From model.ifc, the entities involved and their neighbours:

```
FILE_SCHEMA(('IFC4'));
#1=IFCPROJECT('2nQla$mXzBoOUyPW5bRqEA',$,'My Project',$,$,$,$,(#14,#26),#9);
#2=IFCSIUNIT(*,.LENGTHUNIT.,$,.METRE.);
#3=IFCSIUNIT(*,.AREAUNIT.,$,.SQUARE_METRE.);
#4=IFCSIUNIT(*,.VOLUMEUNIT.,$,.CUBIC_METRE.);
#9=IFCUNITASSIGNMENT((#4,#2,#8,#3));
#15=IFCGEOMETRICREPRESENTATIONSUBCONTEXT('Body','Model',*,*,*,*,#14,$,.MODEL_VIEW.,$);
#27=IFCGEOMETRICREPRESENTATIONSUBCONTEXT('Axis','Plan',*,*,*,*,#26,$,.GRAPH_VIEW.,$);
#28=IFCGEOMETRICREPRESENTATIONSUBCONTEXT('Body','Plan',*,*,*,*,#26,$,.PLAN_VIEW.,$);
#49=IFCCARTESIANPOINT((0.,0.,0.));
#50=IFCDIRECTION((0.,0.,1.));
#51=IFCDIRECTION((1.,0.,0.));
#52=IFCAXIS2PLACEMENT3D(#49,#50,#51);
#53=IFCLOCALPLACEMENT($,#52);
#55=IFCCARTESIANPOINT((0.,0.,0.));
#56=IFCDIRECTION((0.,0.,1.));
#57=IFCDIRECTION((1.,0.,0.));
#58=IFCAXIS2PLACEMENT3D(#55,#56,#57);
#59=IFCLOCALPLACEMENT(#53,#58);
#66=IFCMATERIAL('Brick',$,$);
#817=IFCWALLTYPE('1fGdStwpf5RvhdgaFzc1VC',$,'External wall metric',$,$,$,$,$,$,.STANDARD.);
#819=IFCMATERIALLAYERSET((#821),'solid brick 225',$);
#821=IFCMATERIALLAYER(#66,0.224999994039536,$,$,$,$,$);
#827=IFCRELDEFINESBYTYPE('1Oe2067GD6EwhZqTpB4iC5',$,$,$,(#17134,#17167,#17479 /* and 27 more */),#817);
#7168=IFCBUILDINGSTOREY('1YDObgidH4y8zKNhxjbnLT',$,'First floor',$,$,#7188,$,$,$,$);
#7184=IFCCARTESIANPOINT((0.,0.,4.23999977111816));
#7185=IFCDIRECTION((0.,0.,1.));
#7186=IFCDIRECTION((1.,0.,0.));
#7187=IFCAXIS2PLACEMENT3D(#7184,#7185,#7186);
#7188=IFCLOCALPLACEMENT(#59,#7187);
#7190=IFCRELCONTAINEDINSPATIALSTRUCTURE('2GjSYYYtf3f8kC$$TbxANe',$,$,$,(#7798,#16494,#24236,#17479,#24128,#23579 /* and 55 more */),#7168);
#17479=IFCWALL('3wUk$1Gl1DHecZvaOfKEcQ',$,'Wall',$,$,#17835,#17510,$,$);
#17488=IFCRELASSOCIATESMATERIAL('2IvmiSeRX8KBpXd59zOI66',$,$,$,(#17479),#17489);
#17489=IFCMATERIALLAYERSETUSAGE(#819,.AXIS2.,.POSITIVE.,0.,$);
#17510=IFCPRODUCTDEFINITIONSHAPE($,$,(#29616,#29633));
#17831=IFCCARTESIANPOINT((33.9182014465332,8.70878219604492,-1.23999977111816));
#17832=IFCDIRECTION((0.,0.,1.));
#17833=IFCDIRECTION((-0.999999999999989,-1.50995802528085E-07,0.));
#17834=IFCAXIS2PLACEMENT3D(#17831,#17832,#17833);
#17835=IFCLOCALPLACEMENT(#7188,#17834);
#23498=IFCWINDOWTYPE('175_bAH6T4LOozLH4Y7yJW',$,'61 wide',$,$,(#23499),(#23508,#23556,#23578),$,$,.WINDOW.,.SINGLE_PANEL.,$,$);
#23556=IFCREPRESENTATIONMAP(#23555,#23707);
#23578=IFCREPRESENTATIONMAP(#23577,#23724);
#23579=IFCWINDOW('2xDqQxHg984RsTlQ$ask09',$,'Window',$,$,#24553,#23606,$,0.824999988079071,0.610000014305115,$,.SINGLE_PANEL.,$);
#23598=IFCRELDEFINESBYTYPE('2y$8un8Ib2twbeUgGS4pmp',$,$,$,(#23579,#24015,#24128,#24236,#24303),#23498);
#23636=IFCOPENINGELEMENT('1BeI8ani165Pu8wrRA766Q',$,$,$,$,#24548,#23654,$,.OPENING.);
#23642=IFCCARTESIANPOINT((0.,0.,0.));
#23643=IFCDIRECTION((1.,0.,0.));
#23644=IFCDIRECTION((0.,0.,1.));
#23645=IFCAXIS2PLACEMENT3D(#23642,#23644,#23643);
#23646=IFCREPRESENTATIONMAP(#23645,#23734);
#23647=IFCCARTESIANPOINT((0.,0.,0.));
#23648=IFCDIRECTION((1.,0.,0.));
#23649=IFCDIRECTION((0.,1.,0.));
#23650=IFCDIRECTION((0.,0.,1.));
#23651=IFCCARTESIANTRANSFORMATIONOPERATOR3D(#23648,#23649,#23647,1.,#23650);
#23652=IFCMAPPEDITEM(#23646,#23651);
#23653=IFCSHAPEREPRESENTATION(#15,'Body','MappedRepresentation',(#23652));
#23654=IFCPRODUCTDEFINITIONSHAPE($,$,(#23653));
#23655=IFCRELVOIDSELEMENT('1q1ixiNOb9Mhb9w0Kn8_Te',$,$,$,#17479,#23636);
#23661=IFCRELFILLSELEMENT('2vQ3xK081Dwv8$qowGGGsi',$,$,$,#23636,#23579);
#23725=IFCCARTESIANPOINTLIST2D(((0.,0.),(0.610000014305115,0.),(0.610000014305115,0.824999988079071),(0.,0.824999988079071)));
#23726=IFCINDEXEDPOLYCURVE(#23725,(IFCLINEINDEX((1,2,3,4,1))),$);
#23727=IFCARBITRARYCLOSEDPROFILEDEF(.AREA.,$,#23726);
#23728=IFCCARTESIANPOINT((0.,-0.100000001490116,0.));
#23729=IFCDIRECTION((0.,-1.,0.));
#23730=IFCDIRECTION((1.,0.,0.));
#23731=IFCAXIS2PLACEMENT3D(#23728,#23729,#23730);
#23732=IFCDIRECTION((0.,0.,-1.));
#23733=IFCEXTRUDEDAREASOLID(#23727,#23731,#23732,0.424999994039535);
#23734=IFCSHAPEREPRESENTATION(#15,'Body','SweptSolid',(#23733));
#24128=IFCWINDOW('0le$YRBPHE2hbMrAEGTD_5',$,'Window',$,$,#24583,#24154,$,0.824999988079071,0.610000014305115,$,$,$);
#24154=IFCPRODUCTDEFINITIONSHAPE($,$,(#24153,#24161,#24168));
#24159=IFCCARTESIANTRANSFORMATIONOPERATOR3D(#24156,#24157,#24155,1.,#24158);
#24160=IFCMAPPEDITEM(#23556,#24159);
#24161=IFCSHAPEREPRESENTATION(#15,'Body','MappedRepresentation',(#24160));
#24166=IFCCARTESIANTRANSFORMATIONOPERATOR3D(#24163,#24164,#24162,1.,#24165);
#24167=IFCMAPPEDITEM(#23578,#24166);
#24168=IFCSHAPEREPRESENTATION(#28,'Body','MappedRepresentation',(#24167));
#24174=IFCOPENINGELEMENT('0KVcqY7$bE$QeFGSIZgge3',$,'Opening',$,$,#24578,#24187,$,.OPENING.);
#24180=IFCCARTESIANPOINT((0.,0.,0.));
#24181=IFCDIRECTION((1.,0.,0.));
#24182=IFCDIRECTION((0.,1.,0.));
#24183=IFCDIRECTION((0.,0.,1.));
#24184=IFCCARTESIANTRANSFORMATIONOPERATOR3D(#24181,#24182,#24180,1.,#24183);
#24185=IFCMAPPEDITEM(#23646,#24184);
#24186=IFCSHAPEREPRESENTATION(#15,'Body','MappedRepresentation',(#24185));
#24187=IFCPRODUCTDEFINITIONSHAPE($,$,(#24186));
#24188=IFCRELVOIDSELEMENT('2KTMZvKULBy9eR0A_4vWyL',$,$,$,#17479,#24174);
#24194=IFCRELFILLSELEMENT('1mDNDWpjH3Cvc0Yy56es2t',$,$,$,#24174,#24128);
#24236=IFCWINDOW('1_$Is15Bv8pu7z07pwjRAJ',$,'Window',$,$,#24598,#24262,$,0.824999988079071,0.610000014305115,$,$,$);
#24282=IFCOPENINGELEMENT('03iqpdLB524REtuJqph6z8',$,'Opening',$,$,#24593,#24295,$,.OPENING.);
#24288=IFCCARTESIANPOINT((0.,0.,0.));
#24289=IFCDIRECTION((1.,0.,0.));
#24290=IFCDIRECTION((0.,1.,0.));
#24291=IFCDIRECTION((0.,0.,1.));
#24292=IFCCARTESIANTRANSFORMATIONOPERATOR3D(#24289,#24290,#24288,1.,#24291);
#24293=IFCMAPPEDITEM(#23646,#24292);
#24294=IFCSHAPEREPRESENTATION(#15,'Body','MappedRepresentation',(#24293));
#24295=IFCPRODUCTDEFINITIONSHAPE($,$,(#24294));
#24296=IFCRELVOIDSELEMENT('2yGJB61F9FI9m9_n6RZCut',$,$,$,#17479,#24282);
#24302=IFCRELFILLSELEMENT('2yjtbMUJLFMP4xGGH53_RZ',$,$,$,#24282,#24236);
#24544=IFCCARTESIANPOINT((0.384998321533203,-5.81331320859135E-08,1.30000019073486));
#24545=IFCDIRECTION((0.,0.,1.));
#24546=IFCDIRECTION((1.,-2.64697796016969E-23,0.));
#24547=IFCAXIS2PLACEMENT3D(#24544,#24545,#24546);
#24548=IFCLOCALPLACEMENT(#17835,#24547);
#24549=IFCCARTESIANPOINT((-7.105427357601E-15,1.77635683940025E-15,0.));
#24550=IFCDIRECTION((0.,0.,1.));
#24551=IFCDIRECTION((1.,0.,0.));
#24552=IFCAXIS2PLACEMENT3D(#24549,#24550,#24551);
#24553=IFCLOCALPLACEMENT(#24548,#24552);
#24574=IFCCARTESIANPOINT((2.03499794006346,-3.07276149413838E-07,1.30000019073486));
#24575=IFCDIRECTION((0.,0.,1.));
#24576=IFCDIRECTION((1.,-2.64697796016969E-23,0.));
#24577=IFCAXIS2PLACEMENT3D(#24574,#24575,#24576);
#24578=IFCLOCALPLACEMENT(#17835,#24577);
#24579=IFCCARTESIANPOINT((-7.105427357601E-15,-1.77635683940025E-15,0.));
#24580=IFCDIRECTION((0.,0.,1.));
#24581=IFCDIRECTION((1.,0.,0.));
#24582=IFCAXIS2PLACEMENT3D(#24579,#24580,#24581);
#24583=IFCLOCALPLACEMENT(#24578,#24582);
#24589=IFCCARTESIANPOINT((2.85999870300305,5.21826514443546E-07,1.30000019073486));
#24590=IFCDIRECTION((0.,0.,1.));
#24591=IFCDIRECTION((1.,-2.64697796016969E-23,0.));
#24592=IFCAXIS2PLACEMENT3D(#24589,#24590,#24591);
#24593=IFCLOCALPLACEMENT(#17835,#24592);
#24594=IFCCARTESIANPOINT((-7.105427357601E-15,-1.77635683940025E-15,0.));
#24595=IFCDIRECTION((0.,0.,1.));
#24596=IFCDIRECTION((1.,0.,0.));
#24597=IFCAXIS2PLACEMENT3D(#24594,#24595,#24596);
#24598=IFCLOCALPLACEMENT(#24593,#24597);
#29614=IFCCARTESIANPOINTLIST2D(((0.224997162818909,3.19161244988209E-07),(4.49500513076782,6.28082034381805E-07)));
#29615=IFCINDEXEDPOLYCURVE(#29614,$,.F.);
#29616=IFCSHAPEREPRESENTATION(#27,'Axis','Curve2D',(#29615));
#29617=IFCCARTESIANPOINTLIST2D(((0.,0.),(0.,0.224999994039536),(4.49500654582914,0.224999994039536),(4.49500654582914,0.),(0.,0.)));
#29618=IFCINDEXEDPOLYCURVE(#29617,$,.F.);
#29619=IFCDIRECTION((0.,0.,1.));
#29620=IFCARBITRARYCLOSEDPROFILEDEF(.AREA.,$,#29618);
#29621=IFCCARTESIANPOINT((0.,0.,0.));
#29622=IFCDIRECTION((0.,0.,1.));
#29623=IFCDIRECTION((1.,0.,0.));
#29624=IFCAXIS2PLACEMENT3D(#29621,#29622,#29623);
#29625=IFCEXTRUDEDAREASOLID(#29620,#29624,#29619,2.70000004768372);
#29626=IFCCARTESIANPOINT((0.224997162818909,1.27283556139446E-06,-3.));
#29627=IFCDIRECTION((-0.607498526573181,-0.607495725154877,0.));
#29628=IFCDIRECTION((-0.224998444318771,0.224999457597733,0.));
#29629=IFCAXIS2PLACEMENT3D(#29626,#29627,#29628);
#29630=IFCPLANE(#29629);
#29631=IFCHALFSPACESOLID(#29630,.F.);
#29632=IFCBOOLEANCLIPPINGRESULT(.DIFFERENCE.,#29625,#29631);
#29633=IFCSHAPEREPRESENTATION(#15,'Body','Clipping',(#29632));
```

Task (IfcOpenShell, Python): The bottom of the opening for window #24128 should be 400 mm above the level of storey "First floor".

```python
import numpy as np
import ifcopenshell
import ifcopenshell.api.geometry
import ifcopenshell.geom
import ifcopenshell.util.element
import ifcopenshell.util.placement
import ifcopenshell.util.shape
import ifcopenshell.util.unit

model = ifcopenshell.open("model.ifc")
unit_scale = ifcopenshell.util.unit.calculate_unit_scale(model)

window = model.by_guid("0le$YRBPHE2hbMrAEGTD_5")
opening = window.FillsVoids[0].RelatingOpeningElement
storey = ifcopenshell.util.element.get_container(window, ifc_class="IfcBuildingStorey")
level = ifcopenshell.util.placement.get_local_placement(storey.ObjectPlacement)[2, 3]

# The opening's origin need not be at the sill, so measure its lowest point.
shape = ifcopenshell.geom.create_shape(ifcopenshell.geom.settings(), opening)
bottom = ifcopenshell.util.shape.get_shape_bottom_elevation(shape, shape.geometry) / unit_scale
dz = level + 0.4 - bottom

shift = np.array([0.0, 0.0, dz])
# The window is placed relative to its opening, so it follows when the opening moves.
matrix = ifcopenshell.util.placement.get_local_placement(opening.ObjectPlacement)
matrix[:3, 3] += shift
ifcopenshell.api.geometry.edit_object_placement(
    model, product=opening, matrix=matrix, is_si=False, should_transform_children=True
)

print(f"moved by {dz * unit_scale:+.3f} m")

model.write("model_edited.ifc")
```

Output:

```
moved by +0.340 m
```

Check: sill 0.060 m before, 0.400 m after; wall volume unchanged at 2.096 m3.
